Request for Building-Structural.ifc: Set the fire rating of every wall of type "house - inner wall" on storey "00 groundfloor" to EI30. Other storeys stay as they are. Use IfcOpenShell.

First a look at what the model holds.

```python
import ifcopenshell
import ifcopenshell.util.element

model = ifcopenshell.open("Building-Structural.ifc")
print(model.schema)
storey = next(s for s in model.by_type("IfcBuildingStorey") if s.Name == "00 groundfloor")
walls = [e for e in ifcopenshell.util.element.get_decomposition(storey) if e.is_a("IfcWall")]
seen = {}
for e in walls:
    element_type = ifcopenshell.util.element.get_type(e)
    key = (element_type.Name if element_type != e and element_type else None, ifcopenshell.util.element.get_pset(e, "Pset_WallCommon", "FireRating"))
    seen[key] = seen.get(key, 0) + 1
for (name, value), count in sorted(seen.items(), key=str):
    print(count, "x", name, "|", value)
```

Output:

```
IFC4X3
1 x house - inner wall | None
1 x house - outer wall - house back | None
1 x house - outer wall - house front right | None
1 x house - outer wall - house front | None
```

```python
import ifcopenshell
import ifcopenshell.api.pset
import ifcopenshell.util.element

model = ifcopenshell.open("Building-Structural.ifc")

storey = next(s for s in model.by_type("IfcBuildingStorey") if s.Name == "00 groundfloor")
walls = [e for e in ifcopenshell.util.element.get_decomposition(storey) if e.is_a("IfcWall")]

count = 0
for e in walls:
    element_type = ifcopenshell.util.element.get_type(e)
    if element_type in (None, e) or element_type.Name != "house - inner wall":
        continue
    # add_pset returns the element's existing set when there is one.
    pset = ifcopenshell.api.pset.add_pset(model, product=e, name="Pset_WallCommon")
    ifcopenshell.api.pset.edit_pset(model, pset=pset, properties={"FireRating": "EI30"})
    count += 1

print(count, "walls updated")

model.write("Building-Structural_v2.ifc")
```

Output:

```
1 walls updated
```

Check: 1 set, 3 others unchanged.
